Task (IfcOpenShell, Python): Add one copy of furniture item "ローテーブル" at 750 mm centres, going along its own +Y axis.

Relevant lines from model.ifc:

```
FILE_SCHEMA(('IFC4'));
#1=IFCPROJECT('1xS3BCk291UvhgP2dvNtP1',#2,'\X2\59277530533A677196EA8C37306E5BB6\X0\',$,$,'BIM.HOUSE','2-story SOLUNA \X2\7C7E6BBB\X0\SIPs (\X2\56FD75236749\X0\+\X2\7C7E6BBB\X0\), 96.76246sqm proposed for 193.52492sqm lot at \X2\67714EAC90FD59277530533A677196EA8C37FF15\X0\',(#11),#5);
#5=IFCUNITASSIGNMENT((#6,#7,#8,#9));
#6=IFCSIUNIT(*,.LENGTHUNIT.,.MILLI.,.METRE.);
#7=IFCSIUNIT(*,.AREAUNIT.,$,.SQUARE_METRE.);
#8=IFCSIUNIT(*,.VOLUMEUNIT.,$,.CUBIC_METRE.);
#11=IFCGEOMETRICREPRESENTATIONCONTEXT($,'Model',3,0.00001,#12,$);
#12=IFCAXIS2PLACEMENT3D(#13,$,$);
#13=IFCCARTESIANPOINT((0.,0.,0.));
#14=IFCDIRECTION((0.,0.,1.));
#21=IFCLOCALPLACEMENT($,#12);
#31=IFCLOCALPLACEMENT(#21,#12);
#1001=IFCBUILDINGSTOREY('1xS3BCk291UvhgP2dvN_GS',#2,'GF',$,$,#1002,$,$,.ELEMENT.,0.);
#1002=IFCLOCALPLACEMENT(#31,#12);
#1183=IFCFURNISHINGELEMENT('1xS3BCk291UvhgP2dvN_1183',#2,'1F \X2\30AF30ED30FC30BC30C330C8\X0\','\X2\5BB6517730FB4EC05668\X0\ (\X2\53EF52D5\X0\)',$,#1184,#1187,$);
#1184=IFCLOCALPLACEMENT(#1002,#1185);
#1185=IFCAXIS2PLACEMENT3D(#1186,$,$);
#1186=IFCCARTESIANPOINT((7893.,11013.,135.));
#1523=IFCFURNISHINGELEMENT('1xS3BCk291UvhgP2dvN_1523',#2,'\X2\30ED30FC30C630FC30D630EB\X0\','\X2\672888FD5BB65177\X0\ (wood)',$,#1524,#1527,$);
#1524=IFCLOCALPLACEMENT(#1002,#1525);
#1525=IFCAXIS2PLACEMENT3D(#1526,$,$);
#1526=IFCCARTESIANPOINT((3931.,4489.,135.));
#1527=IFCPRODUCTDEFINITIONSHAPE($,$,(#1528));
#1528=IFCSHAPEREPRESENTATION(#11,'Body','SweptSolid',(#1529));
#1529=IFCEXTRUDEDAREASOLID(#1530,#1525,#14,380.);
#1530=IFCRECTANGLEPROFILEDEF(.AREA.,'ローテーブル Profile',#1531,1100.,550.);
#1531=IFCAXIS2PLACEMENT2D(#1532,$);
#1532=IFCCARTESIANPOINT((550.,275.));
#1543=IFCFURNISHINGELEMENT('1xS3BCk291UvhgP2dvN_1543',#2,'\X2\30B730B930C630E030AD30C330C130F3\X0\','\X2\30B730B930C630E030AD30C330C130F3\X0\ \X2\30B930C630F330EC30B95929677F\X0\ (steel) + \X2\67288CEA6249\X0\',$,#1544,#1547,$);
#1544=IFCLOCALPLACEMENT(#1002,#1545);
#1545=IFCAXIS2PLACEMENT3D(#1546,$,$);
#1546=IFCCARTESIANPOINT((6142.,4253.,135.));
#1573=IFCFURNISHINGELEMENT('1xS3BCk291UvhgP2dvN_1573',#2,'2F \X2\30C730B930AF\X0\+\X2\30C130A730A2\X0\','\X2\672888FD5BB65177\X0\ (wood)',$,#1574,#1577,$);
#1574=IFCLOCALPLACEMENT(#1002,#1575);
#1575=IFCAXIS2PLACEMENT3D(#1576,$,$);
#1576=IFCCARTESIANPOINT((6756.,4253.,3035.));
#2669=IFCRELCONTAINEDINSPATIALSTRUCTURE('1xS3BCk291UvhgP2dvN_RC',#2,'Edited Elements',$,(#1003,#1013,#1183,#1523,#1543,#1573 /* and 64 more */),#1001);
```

```python
import ifcopenshell
import ifcopenshell.api.geometry
import ifcopenshell.api.root
import ifcopenshell.util.element
import ifcopenshell.util.placement
import ifcopenshell.util.unit

model = ifcopenshell.open("model.ifc")
unit_scale = ifcopenshell.util.unit.calculate_unit_scale(model)


def reuse_history(source, copy):
    """copy_class also copies each property set's owner history, people and application; keep the originals."""
    for rel in copy.IsDefinedBy:
        if rel.is_a("IfcRelDefinesByProperties") and (history := rel.RelatingPropertyDefinition.OwnerHistory):
            rel.RelatingPropertyDefinition.OwnerHistory = source.OwnerHistory
            ifcopenshell.util.element.remove_deep2(model, history)


source = model.by_guid("1xS3BCk291UvhgP2dvN_1523")
base = ifcopenshell.util.placement.get_local_placement(source.ObjectPlacement)
step = base[:3, 1] * 0.75 / unit_scale

for i in range(1, 2):
    copy = ifcopenshell.api.root.copy_class(model, product=source)
    copy.Representation = ifcopenshell.util.element.copy_deep(
        model, source.Representation, exclude=["IfcGeometricRepresentationContext", "IfcRepresentationMap"]
    )
    reuse_history(source, copy)
    matrix = base.copy()
    matrix[:3, 3] += i * step
    print("added at", matrix[:3, 3].round(3) + 0.0)
    ifcopenshell.api.geometry.edit_object_placement(model, product=copy, matrix=matrix, is_si=False)

model.write("model_v2.ifc")
```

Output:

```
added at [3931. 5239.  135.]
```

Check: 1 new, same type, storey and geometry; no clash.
